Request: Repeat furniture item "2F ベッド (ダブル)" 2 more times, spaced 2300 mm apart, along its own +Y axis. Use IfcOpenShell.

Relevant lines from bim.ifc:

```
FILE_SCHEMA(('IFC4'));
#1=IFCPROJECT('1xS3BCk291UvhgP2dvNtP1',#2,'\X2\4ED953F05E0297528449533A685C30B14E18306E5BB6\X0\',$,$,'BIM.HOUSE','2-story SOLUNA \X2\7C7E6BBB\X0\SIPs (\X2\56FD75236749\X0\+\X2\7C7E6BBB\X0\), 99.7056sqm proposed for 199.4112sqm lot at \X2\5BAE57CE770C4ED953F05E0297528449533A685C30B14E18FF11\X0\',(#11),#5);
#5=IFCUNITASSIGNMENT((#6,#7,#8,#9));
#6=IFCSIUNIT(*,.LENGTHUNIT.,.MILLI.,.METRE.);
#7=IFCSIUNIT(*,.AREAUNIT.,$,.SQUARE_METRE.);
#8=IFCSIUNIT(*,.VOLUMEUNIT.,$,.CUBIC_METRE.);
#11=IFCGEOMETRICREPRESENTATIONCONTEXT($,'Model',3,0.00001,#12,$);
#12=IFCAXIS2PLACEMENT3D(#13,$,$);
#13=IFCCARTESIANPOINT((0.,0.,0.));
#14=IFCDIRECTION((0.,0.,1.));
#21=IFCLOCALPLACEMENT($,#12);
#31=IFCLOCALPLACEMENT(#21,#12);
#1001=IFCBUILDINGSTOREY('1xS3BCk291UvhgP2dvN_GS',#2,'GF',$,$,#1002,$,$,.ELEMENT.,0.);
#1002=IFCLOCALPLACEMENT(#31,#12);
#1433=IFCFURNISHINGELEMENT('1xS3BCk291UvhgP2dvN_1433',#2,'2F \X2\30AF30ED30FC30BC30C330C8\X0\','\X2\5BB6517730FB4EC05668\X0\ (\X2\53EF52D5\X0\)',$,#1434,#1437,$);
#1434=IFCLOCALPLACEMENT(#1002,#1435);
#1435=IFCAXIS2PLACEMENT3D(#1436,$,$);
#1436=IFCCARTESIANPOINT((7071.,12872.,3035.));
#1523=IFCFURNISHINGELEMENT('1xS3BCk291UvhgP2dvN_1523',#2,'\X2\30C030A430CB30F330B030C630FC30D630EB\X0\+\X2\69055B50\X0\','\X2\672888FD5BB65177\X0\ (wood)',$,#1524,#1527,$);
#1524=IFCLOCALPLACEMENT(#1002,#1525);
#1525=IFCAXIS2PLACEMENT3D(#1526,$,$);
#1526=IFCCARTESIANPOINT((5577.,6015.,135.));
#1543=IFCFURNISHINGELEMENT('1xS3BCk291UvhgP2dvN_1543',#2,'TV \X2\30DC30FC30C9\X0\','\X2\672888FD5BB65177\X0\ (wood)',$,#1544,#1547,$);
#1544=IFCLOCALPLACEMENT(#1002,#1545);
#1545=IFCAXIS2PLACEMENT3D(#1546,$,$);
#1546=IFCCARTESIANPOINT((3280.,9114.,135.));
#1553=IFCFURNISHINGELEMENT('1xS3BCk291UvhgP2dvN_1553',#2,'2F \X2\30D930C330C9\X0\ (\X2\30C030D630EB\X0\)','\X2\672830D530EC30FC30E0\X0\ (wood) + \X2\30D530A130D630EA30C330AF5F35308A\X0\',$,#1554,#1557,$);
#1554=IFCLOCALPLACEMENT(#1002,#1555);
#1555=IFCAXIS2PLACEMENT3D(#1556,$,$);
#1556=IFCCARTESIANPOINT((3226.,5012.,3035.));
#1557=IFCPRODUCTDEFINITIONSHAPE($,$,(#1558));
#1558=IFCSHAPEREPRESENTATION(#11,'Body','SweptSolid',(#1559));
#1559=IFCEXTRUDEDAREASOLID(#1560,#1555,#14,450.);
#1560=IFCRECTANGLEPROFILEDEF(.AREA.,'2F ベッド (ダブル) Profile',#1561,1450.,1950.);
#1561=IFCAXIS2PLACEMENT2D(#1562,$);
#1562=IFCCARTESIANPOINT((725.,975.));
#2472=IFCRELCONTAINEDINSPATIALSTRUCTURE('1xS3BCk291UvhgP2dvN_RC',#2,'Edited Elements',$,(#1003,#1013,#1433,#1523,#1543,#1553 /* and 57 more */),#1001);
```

```python
import ifcopenshell
import ifcopenshell.api.geometry
import ifcopenshell.api.root
import ifcopenshell.util.element
import ifcopenshell.util.placement
import ifcopenshell.util.unit

model = ifcopenshell.open("bim.ifc")
unit_scale = ifcopenshell.util.unit.calculate_unit_scale(model)


def reuse_history(source, copy):
    """copy_class also copies each property set's owner history, people and application; keep the originals."""
    for rel in copy.IsDefinedBy:
        if rel.is_a("IfcRelDefinesByProperties") and (history := rel.RelatingPropertyDefinition.OwnerHistory):
            rel.RelatingPropertyDefinition.OwnerHistory = source.OwnerHistory
            ifcopenshell.util.element.remove_deep2(model, history)


source = model.by_guid("1xS3BCk291UvhgP2dvN_1553")
base = ifcopenshell.util.placement.get_local_placement(source.ObjectPlacement)
step = base[:3, 1] * 2.3 / unit_scale

for i in range(1, 3):
    copy = ifcopenshell.api.root.copy_class(model, product=source)
    copy.Representation = ifcopenshell.util.element.copy_deep(
        model, source.Representation, exclude=["IfcGeometricRepresentationContext", "IfcRepresentationMap"]
    )
    reuse_history(source, copy)
    matrix = base.copy()
    matrix[:3, 3] += i * step
    print("added at", matrix[:3, 3].round(3) + 0.0)
    ifcopenshell.api.geometry.edit_object_placement(model, product=copy, matrix=matrix, is_si=False)

model.write("bim_v2.ifc")
```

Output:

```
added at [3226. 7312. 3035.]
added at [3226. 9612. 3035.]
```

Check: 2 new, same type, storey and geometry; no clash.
